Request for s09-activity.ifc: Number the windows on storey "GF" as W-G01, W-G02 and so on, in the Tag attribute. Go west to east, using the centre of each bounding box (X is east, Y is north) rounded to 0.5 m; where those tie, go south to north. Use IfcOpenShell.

First a look at what the model holds.

```python
import ifcopenshell
import ifcopenshell.util.element
import ifcopenshell.util.placement

model = ifcopenshell.open("s09-activity.ifc")
print(model.schema)
storey = next(s for s in model.by_type("IfcBuildingStorey") if s.Name == "GF")
windows = [e for e in ifcopenshell.util.element.get_decomposition(storey) if e.is_a("IfcWindow")]
for e in sorted(windows, key=lambda e: e.id()):
    origin = ifcopenshell.util.placement.get_local_placement(e.ObjectPlacement)[:3, 3]
    print(e.id(), e.Tag, e.Name, origin.round(2) + 0.0, sep=" | ")
```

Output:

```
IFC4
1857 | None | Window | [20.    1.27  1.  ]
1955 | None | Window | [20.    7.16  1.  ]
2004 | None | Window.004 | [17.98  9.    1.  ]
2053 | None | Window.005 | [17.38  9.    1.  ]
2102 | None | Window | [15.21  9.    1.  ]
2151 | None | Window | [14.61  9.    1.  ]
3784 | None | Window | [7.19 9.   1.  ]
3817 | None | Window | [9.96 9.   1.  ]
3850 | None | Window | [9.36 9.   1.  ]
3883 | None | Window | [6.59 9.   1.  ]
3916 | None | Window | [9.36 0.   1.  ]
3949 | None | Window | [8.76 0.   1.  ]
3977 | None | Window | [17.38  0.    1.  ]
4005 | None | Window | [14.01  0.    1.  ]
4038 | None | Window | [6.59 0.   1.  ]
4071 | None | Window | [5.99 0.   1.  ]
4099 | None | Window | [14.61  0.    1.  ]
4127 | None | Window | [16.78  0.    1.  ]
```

```python
import ifcopenshell
import ifcopenshell.geom
import ifcopenshell.util.element
import ifcopenshell.util.shape

model = ifcopenshell.open("s09-activity.ifc")
settings = ifcopenshell.geom.settings()
settings.set("use-world-coords", True)


def centre(element):
    shape = ifcopenshell.geom.create_shape(settings, element)
    return ifcopenshell.util.shape.get_bbox_centroid(shape.geometry)


storey = next(s for s in model.by_type("IfcBuildingStorey") if s.Name == "GF")
windows = [e for e in ifcopenshell.util.element.get_decomposition(storey) if e.is_a("IfcWindow")]

# Insertion points can sit at a corner or the storey origin, so sort by the geometry (in metres).
centres = {e: centre(e) for e in windows}
windows.sort(key=lambda e: (round(centres[e][0] / 0.5), centres[e][1]))

for i, e in enumerate(windows, start=1):
    number = f"W-G{i:02d}"
    e.Tag = number
    print(e.id(), number)

model.write("s09-activity_updated.ifc")
```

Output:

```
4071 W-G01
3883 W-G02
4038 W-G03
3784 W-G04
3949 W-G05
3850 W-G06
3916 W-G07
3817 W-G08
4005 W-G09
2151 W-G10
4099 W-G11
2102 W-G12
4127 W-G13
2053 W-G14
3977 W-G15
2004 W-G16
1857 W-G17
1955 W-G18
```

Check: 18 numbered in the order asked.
